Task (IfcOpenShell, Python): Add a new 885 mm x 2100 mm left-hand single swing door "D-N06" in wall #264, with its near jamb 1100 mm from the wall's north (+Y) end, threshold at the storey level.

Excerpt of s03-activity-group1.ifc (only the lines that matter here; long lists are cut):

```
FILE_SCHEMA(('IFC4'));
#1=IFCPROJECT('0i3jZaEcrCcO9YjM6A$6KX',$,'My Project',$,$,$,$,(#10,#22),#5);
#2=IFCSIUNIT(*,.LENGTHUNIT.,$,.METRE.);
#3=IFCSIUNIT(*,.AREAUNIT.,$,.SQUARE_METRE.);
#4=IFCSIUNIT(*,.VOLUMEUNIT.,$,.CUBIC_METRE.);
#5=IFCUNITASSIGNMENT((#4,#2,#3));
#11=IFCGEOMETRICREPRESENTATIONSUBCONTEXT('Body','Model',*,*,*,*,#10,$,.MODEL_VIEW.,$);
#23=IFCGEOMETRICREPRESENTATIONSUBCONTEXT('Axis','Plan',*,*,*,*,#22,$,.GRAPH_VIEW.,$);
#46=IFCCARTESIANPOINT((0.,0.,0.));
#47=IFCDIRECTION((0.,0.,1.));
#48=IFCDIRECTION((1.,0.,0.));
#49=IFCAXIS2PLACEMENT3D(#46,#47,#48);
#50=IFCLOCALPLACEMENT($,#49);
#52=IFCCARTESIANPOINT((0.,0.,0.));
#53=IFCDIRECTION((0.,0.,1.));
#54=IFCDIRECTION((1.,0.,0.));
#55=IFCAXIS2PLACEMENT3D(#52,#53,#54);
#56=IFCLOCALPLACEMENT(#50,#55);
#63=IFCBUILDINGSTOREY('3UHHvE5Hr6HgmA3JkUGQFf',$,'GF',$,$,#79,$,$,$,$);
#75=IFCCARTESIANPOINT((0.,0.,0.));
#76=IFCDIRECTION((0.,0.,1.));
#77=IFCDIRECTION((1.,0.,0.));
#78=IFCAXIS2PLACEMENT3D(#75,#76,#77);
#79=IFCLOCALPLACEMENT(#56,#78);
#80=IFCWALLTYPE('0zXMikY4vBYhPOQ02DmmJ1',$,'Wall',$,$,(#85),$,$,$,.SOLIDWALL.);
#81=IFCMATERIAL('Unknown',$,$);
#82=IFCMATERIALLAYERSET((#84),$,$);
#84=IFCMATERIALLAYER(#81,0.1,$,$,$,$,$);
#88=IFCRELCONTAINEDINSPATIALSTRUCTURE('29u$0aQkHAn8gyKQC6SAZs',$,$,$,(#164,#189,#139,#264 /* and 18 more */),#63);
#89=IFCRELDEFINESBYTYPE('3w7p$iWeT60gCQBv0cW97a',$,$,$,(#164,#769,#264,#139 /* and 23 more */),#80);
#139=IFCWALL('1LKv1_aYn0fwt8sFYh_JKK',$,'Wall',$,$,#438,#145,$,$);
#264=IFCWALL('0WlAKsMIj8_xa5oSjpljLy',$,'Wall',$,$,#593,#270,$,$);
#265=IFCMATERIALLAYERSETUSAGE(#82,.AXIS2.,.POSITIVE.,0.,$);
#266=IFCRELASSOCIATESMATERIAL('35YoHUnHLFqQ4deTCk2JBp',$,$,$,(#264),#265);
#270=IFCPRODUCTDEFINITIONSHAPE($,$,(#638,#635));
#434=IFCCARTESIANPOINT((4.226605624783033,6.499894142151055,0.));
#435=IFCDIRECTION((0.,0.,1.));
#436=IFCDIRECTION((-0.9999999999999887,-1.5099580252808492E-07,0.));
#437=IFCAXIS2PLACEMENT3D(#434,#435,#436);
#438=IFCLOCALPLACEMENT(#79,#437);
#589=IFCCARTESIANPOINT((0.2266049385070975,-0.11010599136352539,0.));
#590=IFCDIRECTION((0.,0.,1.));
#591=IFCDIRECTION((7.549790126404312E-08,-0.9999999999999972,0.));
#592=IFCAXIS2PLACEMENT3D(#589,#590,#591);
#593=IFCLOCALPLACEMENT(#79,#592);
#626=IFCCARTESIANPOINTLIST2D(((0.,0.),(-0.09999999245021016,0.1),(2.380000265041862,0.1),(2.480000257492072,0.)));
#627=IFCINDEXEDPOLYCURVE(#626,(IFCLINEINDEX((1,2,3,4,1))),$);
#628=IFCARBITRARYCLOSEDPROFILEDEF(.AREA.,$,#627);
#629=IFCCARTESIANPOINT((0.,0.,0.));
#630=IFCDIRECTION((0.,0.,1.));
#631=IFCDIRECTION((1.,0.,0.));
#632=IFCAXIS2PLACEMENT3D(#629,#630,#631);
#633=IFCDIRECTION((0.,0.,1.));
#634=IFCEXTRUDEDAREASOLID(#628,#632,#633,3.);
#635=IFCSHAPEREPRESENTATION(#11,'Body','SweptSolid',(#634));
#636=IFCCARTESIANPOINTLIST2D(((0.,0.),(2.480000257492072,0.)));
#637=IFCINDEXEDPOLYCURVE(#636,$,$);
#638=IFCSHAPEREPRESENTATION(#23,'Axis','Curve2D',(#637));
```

```python
import numpy as np
import ifcopenshell
import ifcopenshell.api.feature
import ifcopenshell.api.geometry
import ifcopenshell.api.root
import ifcopenshell.api.spatial
import ifcopenshell.geom
import ifcopenshell.util.element
import ifcopenshell.util.placement
import ifcopenshell.util.representation
import ifcopenshell.util.shape
import ifcopenshell.util.unit

model = ifcopenshell.open("s03-activity-group1.ifc")
unit_scale = ifcopenshell.util.unit.calculate_unit_scale(model)
settings = ifcopenshell.geom.settings()


def volume(element):
    """Net volume in cubic metres, openings subtracted."""
    shape = ifcopenshell.geom.create_shape(settings, element)
    return ifcopenshell.util.shape.get_volume(shape.geometry)


wall = model.by_id(264)
storey = ifcopenshell.util.element.get_container(wall, ifc_class="IfcBuildingStorey")
context = ifcopenshell.util.representation.get_context(model, "Model", "Body", "MODEL_VIEW")
before = volume(wall)

width, height, from_end, sill = 0.885, 2.1, 1.1, 0.0  # metres

# The wall runs along its own X axis, and the end named is its -X end.
wall_shape = ifcopenshell.geom.create_shape(settings, wall)
x, y, z = ifcopenshell.util.shape.get_vertices(wall_shape.geometry).T
start = x.min() + from_end
face, thickness = float(y.min()), float(y.max() - y.min())
wall_matrix = ifcopenshell.util.placement.get_local_placement(wall.ObjectPlacement)
level = ifcopenshell.util.placement.get_local_placement(storey.ObjectPlacement)[2, 3]


def in_wall(x, y):
    """Placement at x, y metres in the wall's axes, at sill height."""
    matrix = wall_matrix.copy()
    matrix[:, 3] = wall_matrix @ np.array([x / unit_scale, y / unit_scale, 0.0, 1.0])
    matrix[2, 3] = level + sill / unit_scale
    return matrix


# Opening: a box that overshoots both wall faces by 50 mm.
opening = ifcopenshell.api.root.create_entity(model, ifc_class="IfcOpeningElement", predefined_type="OPENING")
box = ifcopenshell.api.geometry.add_wall_representation(
    model, context=context, length=width, height=height, thickness=thickness + 0.1
)
ifcopenshell.api.geometry.assign_representation(model, product=opening, representation=box)
ifcopenshell.api.geometry.edit_object_placement(model, product=opening, matrix=in_wall(start, face - 0.05), is_si=False)
ifcopenshell.api.feature.add_feature(model, feature=opening, element=wall)

door = ifcopenshell.api.root.create_entity(model, ifc_class="IfcDoor", name="D-N06", predefined_type="DOOR")
door.OverallWidth, door.OverallHeight = width / unit_scale, height / unit_scale
door.OperationType = "SINGLE_SWING_LEFT"
body = ifcopenshell.api.geometry.add_door_representation(
    model,
    context=context,
    overall_width=door.OverallWidth,
    overall_height=door.OverallHeight,
    operation_type="SINGLE_SWING_LEFT",
    lining_properties={"LiningDepth": thickness / unit_scale, "ThresholdDepth": thickness / unit_scale},
)
ifcopenshell.api.geometry.assign_representation(model, product=door, representation=body)
ifcopenshell.api.spatial.assign_container(model, products=[door], relating_structure=storey)
ifcopenshell.api.feature.add_filling(model, opening=opening, element=door)

# The lining spans the wall, so the door starts at the wall face.
ifcopenshell.api.geometry.edit_object_placement(model, product=door, matrix=in_wall(start, face), is_si=False)

after = volume(wall)

print(f"wall volume {before:.3f} -> {after:.3f} m3")

model.write("s03-activity-group1_v2.ifc")
```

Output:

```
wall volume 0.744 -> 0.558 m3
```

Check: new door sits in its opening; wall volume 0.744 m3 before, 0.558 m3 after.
